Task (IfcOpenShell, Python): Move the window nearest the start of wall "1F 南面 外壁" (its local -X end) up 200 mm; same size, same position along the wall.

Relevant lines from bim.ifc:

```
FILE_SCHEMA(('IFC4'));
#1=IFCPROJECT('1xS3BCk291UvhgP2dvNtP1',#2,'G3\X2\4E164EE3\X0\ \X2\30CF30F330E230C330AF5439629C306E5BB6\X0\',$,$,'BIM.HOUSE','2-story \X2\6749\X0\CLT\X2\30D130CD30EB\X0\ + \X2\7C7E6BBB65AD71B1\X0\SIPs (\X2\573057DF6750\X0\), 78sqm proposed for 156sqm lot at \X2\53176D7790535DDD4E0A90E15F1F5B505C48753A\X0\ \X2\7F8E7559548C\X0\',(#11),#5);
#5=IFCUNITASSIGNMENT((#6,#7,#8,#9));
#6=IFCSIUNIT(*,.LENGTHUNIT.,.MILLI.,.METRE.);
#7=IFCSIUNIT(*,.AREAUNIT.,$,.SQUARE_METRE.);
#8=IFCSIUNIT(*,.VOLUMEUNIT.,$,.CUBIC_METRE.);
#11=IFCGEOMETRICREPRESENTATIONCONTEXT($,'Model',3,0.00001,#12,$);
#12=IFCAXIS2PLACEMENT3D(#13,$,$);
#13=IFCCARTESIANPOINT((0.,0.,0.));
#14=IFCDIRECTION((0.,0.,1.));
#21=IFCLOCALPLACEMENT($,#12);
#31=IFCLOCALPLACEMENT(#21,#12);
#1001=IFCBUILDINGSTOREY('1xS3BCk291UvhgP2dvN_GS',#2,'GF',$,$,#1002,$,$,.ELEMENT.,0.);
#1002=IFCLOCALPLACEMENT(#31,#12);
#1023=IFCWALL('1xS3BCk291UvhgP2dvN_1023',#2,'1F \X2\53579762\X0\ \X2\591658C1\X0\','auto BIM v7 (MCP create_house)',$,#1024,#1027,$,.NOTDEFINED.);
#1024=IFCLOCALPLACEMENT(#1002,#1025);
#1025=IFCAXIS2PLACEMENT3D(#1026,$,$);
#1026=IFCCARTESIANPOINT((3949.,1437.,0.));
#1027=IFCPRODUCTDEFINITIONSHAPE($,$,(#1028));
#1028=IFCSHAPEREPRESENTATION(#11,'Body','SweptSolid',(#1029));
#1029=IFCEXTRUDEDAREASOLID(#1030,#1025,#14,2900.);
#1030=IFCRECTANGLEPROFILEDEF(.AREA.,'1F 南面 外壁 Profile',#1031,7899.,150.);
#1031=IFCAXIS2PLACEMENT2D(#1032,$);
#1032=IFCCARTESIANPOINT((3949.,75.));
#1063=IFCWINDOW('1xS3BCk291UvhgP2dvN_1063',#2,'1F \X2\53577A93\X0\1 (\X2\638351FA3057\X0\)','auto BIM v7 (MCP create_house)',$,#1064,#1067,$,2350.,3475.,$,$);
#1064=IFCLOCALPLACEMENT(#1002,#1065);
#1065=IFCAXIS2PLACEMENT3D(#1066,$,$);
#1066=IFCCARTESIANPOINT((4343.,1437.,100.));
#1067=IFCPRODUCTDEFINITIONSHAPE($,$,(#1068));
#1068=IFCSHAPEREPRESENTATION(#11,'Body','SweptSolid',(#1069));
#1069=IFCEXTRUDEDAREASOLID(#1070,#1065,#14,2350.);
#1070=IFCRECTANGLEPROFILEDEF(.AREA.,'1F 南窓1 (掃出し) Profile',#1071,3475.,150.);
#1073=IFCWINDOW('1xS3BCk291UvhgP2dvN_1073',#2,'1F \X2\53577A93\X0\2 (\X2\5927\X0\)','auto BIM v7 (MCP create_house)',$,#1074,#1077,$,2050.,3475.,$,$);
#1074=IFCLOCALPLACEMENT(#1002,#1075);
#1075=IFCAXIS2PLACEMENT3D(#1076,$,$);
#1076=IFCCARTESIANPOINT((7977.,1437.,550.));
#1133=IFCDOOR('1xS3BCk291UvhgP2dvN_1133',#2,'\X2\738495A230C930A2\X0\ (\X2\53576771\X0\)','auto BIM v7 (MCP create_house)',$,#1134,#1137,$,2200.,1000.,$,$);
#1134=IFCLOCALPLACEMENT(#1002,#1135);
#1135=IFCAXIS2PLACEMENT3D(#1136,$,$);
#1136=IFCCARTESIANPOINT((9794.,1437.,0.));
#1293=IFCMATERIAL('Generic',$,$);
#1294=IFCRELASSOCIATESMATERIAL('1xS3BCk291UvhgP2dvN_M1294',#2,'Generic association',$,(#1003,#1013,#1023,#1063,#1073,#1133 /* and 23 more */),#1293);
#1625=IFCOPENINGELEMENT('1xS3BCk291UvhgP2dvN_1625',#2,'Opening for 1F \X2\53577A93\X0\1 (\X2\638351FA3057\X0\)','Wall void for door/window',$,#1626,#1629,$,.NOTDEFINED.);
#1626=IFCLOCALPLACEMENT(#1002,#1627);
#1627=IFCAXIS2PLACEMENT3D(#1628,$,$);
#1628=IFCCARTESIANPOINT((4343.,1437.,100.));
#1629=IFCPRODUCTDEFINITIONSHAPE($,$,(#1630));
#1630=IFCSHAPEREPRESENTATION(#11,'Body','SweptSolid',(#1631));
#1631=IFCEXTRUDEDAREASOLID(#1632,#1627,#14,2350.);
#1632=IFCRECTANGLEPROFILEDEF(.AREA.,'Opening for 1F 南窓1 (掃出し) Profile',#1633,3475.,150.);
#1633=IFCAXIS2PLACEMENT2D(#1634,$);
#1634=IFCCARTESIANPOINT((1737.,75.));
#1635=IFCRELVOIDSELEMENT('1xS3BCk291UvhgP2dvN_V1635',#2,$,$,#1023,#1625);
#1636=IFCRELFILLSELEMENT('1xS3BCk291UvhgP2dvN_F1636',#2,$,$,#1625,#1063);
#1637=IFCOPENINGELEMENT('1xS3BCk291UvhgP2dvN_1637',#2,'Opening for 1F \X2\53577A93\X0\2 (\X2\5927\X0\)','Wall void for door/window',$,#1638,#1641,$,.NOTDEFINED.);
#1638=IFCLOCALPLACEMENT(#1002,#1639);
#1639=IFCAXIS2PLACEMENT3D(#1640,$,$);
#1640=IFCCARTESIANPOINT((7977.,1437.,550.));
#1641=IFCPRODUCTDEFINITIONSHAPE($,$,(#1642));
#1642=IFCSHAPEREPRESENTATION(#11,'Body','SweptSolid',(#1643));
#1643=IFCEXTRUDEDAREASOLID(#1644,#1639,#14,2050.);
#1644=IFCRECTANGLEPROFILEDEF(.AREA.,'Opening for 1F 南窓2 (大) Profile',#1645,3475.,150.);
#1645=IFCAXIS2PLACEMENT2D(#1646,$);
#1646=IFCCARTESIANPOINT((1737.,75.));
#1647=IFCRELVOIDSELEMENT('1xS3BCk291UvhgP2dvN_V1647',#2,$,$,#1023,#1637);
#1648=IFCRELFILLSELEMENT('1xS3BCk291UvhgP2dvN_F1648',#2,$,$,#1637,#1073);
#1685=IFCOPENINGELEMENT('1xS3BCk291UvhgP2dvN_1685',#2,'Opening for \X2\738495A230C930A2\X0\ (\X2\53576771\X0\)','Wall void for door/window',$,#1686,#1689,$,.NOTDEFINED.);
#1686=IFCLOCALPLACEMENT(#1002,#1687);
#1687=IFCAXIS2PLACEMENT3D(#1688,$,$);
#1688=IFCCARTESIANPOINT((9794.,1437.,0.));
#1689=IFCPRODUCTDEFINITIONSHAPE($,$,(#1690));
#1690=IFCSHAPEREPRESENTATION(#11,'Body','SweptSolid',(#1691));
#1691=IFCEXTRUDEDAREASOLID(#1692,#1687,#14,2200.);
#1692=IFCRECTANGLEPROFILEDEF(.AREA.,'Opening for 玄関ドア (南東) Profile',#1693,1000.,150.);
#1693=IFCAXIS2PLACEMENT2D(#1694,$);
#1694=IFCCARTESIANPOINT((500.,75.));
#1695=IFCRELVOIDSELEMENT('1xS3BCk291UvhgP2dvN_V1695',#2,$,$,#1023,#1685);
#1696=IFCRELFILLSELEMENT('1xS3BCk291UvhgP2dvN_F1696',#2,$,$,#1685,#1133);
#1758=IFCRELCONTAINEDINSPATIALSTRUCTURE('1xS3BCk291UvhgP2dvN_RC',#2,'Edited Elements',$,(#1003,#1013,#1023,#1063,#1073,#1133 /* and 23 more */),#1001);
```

```python
import numpy as np
import ifcopenshell
import ifcopenshell.api.geometry
import ifcopenshell.util.placement
import ifcopenshell.util.unit

model = ifcopenshell.open("bim.ifc")
unit_scale = ifcopenshell.util.unit.calculate_unit_scale(model)

window = model.by_guid("1xS3BCk291UvhgP2dvN_1063")
opening = window.FillsVoids[0].RelatingOpeningElement
dz = 0.2 / unit_scale

shift = np.array([0.0, 0.0, dz])
# The window is not placed relative to its opening, so move both.
for product in (opening, window):
    matrix = ifcopenshell.util.placement.get_local_placement(product.ObjectPlacement)
    matrix[:3, 3] += shift
    ifcopenshell.api.geometry.edit_object_placement(model, product=product, matrix=matrix, is_si=False)

print(f"moved by {dz * unit_scale:+.3f} m")

model.write("bim-out.ifc")
```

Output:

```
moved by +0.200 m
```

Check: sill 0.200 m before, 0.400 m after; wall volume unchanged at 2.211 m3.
